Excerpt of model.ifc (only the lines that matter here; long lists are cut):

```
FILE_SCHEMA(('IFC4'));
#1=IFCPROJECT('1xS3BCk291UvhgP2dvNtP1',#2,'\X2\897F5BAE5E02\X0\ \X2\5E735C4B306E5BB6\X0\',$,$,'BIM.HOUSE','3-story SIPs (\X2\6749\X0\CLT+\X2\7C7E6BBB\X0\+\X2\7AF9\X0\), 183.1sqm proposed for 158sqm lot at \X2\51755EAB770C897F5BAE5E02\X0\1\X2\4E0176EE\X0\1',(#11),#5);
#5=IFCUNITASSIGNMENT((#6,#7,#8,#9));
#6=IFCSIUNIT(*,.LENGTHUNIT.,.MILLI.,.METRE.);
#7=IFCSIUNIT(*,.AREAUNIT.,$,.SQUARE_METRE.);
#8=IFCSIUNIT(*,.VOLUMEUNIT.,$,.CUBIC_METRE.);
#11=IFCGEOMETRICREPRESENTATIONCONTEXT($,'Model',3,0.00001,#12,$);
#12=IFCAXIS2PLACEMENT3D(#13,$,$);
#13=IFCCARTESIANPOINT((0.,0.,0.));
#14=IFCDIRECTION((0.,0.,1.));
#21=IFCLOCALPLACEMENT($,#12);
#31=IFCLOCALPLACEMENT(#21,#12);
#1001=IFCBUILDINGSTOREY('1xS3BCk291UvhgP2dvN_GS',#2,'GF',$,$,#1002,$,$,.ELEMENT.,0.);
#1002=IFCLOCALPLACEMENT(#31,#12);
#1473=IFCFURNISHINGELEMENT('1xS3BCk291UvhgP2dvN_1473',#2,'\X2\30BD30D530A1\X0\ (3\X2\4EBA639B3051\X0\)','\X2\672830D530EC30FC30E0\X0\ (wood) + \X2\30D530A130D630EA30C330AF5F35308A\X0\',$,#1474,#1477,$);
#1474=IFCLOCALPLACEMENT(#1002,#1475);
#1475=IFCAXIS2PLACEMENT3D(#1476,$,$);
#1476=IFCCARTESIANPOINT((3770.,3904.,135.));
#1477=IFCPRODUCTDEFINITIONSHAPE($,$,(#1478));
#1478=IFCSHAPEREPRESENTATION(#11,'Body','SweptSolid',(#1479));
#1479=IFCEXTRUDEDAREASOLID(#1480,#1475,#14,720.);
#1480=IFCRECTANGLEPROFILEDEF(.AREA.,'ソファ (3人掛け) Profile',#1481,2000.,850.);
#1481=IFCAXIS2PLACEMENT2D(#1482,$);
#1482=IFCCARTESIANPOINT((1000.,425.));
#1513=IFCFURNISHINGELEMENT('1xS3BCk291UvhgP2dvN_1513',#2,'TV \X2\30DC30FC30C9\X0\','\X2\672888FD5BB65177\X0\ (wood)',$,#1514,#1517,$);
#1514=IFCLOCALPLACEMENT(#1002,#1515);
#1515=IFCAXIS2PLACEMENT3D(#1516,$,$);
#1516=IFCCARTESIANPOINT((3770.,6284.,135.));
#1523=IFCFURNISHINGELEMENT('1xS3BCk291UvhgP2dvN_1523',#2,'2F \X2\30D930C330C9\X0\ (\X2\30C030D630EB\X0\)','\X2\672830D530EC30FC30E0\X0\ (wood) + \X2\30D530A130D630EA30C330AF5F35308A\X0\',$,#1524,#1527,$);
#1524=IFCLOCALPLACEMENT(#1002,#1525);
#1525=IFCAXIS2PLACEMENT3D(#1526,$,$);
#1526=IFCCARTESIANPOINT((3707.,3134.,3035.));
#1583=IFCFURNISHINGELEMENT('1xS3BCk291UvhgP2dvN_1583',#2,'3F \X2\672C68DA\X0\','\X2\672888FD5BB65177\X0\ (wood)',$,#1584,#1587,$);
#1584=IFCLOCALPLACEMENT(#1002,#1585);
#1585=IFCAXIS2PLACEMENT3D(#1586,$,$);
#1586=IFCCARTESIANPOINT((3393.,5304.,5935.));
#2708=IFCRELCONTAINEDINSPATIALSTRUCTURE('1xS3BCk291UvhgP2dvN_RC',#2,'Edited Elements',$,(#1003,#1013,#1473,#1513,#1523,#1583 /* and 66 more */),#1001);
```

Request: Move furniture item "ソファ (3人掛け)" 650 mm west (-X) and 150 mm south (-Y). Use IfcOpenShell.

```python
import ifcopenshell
import ifcopenshell.api.geometry
import ifcopenshell.util.placement
import ifcopenshell.util.unit

model = ifcopenshell.open("model.ifc")
unit_scale = ifcopenshell.util.unit.calculate_unit_scale(model)

item = model.by_guid("1xS3BCk291UvhgP2dvN_1473")
matrix = ifcopenshell.util.placement.get_local_placement(item.ObjectPlacement)
matrix[0, 3] -= 0.65 / unit_scale
matrix[1, 3] -= 0.15 / unit_scale
ifcopenshell.api.geometry.edit_object_placement(model, product=item, matrix=matrix, is_si=False)

print(ifcopenshell.util.placement.get_local_placement(item.ObjectPlacement).round(3) + 0.0)

model.write("model_edited.ifc")
```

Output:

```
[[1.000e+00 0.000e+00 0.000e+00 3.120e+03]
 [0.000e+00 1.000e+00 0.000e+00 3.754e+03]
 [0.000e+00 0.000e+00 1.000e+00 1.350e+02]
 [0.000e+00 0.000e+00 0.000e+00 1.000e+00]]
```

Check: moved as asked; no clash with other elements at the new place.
